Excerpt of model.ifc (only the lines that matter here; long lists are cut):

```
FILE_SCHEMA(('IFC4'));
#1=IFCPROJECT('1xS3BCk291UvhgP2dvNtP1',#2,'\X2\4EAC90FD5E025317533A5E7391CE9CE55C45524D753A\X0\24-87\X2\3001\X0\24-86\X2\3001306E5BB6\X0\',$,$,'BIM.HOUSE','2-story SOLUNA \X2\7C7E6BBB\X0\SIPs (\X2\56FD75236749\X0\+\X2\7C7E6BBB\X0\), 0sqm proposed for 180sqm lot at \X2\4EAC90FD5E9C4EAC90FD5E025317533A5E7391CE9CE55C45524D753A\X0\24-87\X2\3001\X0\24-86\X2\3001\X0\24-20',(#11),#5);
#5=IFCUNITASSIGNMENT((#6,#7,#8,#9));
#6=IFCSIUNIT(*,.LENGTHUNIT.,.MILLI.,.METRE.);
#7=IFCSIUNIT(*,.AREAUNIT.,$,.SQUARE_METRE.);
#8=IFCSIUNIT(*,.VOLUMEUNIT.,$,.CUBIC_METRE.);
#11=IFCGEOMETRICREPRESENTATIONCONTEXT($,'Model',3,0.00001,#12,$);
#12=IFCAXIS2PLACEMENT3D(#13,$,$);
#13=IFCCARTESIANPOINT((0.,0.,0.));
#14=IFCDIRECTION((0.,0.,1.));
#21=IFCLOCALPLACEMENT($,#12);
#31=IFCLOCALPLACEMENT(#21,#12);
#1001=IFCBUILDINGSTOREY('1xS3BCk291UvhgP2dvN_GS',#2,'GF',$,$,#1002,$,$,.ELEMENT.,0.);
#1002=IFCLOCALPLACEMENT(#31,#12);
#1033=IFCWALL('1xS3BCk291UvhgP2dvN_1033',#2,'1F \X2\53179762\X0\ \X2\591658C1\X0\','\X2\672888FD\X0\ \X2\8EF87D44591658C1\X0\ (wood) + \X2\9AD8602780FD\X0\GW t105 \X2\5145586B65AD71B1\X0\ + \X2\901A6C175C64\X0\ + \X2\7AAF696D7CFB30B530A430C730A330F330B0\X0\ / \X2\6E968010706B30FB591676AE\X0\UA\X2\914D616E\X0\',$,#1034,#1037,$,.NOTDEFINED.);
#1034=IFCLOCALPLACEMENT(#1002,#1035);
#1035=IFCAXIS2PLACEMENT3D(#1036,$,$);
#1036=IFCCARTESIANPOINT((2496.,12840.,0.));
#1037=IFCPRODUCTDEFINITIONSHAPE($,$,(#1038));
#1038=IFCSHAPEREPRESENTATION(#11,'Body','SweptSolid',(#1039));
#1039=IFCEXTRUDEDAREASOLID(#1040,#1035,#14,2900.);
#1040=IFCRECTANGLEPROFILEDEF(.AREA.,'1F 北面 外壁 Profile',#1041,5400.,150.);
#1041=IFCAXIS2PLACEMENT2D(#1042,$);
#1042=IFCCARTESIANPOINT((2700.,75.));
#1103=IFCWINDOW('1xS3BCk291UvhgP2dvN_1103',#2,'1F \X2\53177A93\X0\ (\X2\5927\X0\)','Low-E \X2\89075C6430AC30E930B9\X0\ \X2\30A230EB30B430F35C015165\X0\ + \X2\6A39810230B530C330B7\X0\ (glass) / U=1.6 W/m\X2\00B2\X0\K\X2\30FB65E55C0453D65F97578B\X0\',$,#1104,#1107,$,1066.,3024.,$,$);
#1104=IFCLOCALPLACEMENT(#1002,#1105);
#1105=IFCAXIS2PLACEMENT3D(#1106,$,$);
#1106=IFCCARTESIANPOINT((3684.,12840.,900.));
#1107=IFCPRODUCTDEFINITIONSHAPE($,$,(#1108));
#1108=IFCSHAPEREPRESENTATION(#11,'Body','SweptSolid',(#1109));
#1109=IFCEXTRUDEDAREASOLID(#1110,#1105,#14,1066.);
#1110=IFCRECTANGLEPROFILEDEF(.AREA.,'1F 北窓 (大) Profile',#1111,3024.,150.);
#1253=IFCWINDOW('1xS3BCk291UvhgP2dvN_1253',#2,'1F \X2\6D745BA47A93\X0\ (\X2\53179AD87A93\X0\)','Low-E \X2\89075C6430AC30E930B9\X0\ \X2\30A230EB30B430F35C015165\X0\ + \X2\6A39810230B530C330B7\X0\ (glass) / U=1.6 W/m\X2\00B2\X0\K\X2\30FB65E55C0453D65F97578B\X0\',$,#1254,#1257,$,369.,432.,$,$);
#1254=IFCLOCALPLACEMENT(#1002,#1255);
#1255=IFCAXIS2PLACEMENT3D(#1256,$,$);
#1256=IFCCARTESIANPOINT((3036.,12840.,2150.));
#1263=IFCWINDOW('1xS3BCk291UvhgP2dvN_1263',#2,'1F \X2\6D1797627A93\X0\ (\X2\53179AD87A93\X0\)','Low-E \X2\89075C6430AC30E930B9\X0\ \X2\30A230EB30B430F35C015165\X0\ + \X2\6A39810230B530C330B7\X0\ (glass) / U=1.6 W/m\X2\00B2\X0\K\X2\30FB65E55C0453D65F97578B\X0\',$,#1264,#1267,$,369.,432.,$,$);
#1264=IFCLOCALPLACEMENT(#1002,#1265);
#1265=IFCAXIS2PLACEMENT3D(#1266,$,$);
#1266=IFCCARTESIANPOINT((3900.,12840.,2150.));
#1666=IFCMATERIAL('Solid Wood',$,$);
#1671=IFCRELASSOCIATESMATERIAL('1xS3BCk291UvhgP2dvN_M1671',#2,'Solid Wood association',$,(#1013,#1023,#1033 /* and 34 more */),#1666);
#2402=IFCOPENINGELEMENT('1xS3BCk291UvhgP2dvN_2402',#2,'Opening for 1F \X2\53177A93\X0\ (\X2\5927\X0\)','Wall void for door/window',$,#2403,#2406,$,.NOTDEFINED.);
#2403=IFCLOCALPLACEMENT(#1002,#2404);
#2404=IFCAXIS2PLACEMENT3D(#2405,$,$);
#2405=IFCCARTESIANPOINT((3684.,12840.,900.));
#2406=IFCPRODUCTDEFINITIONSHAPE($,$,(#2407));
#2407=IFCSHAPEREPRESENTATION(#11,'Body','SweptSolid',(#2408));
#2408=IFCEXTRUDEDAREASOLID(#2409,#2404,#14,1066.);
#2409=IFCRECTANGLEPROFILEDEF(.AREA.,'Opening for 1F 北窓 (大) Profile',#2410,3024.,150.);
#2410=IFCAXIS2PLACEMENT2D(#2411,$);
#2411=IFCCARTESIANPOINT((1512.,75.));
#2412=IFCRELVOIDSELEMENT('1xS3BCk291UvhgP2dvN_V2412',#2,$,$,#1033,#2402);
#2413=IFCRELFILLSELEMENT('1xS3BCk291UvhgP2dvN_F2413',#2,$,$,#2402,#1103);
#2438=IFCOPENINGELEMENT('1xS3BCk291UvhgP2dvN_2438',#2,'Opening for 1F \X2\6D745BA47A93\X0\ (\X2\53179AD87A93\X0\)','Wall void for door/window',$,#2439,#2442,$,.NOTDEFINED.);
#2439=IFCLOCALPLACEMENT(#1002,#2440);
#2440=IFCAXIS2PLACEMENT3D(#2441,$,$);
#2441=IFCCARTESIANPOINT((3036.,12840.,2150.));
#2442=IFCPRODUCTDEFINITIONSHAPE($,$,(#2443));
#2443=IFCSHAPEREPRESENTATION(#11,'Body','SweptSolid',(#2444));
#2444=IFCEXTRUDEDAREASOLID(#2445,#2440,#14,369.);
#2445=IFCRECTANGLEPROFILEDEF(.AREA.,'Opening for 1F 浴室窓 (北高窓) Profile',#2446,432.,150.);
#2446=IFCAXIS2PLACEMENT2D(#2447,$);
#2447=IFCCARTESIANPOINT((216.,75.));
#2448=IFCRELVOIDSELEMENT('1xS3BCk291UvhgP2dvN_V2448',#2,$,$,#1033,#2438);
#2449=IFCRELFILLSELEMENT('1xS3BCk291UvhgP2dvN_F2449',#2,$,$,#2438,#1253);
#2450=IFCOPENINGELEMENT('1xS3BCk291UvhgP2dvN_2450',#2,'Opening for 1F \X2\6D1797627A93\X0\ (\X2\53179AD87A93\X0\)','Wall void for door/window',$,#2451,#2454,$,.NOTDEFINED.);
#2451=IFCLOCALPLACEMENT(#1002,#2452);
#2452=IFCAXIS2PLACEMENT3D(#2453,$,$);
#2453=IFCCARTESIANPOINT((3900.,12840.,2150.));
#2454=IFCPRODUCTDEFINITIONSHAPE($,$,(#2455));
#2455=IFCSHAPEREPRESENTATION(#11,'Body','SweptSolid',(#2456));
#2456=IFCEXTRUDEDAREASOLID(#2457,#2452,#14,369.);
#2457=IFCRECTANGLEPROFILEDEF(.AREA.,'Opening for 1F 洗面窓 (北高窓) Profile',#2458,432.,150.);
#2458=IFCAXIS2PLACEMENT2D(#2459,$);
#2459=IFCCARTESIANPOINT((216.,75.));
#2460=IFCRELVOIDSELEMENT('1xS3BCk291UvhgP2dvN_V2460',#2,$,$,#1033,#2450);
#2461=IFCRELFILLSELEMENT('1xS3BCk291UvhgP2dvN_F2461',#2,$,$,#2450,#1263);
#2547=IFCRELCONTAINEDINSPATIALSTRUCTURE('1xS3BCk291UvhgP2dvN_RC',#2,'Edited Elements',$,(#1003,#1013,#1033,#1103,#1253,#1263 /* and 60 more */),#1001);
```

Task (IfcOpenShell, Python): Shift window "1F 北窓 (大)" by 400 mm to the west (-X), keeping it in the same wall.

```python
import ifcopenshell
import ifcopenshell.api.geometry
import ifcopenshell.util.placement

model = ifcopenshell.open("model.ifc")

window = model.by_guid("1xS3BCk291UvhgP2dvN_1103")
opening = window.FillsVoids[0].RelatingOpeningElement
wall = opening.VoidsElements[0].RelatingBuildingElement

wall_matrix = ifcopenshell.util.placement.get_local_placement(wall.ObjectPlacement)
shift = wall_matrix[:3, 0] * -400.0
before = ifcopenshell.util.placement.get_local_placement(window.ObjectPlacement)[:3, 3].copy()

# The window is not placed relative to its opening, so move both.
for product in (opening, window):
    matrix = ifcopenshell.util.placement.get_local_placement(product.ObjectPlacement)
    matrix[:3, 3] += shift
    ifcopenshell.api.geometry.edit_object_placement(model, product=product, matrix=matrix, is_si=False)

after = ifcopenshell.util.placement.get_local_placement(window.ObjectPlacement)[:3, 3]
print("window moved by", (after - before).round(3) + 0.0)

model.write("model-out.ifc")
```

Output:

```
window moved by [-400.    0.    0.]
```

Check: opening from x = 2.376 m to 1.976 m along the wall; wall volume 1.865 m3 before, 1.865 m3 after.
